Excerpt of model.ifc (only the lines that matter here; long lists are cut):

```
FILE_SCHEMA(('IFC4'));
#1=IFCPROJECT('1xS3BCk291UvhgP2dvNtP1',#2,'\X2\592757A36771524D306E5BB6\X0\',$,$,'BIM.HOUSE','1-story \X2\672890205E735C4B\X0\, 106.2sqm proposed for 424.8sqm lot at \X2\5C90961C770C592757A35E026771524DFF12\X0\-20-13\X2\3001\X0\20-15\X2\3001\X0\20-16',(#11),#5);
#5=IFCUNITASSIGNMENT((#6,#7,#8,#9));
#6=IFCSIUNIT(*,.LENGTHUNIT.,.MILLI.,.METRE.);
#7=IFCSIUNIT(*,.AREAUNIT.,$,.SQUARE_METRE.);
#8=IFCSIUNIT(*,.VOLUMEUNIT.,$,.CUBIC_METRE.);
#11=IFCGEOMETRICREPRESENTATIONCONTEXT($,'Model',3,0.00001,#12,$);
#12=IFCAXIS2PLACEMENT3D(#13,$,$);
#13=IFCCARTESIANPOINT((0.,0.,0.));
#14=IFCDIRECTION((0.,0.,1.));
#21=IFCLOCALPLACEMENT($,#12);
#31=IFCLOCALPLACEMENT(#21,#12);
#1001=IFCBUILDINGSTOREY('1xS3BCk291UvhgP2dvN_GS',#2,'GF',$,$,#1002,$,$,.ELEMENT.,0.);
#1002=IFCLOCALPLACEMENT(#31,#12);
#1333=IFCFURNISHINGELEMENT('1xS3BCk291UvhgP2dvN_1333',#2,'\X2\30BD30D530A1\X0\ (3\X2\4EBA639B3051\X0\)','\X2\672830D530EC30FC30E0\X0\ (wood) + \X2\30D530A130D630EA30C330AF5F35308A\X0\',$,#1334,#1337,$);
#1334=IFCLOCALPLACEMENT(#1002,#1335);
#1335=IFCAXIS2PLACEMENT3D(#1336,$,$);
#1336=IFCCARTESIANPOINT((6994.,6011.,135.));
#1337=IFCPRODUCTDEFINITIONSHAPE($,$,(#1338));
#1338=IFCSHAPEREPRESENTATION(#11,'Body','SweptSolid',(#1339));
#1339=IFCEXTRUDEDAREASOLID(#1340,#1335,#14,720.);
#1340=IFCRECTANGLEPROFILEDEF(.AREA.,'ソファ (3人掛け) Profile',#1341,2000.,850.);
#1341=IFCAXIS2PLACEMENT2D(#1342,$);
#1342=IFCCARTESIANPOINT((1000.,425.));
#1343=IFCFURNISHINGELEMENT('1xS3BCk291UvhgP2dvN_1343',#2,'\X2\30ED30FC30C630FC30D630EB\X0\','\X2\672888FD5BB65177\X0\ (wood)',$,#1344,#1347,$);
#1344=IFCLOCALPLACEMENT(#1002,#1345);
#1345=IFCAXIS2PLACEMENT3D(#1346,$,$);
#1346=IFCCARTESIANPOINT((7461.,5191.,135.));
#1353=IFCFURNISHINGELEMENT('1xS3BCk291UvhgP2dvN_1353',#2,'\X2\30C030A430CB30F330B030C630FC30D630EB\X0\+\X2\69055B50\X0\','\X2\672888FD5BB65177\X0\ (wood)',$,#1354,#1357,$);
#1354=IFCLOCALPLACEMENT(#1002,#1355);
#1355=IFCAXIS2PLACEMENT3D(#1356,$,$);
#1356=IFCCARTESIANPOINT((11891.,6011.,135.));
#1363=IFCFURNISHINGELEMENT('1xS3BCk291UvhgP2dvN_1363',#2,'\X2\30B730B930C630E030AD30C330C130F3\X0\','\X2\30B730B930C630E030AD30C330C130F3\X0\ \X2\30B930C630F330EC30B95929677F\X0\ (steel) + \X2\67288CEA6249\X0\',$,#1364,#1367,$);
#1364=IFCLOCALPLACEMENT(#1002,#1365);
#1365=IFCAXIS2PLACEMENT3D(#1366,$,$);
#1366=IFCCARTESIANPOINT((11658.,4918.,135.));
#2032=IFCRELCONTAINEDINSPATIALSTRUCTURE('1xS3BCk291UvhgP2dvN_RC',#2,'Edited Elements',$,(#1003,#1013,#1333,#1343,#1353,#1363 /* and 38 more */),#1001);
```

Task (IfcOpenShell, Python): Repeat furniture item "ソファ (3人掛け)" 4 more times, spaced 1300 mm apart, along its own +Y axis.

```python
import ifcopenshell
import ifcopenshell.api.geometry
import ifcopenshell.api.root
import ifcopenshell.util.element
import ifcopenshell.util.placement
import ifcopenshell.util.unit

model = ifcopenshell.open("model.ifc")
unit_scale = ifcopenshell.util.unit.calculate_unit_scale(model)


def reuse_history(source, copy):
    """copy_class also copies each property set's owner history, people and application; keep the originals."""
    for rel in copy.IsDefinedBy:
        if rel.is_a("IfcRelDefinesByProperties") and (history := rel.RelatingPropertyDefinition.OwnerHistory):
            rel.RelatingPropertyDefinition.OwnerHistory = source.OwnerHistory
            ifcopenshell.util.element.remove_deep2(model, history)


source = model.by_guid("1xS3BCk291UvhgP2dvN_1333")
base = ifcopenshell.util.placement.get_local_placement(source.ObjectPlacement)
step = base[:3, 1] * 1.3 / unit_scale

for i in range(1, 5):
    copy = ifcopenshell.api.root.copy_class(model, product=source)
    copy.Representation = ifcopenshell.util.element.copy_deep(
        model, source.Representation, exclude=["IfcGeometricRepresentationContext", "IfcRepresentationMap"]
    )
    reuse_history(source, copy)
    matrix = base.copy()
    matrix[:3, 3] += i * step
    print("added at", matrix[:3, 3].round(3) + 0.0)
    ifcopenshell.api.geometry.edit_object_placement(model, product=copy, matrix=matrix, is_si=False)

model.write("model_edited.ifc")
```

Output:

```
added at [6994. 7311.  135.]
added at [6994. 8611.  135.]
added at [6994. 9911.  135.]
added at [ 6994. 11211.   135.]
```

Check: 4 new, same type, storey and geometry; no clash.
